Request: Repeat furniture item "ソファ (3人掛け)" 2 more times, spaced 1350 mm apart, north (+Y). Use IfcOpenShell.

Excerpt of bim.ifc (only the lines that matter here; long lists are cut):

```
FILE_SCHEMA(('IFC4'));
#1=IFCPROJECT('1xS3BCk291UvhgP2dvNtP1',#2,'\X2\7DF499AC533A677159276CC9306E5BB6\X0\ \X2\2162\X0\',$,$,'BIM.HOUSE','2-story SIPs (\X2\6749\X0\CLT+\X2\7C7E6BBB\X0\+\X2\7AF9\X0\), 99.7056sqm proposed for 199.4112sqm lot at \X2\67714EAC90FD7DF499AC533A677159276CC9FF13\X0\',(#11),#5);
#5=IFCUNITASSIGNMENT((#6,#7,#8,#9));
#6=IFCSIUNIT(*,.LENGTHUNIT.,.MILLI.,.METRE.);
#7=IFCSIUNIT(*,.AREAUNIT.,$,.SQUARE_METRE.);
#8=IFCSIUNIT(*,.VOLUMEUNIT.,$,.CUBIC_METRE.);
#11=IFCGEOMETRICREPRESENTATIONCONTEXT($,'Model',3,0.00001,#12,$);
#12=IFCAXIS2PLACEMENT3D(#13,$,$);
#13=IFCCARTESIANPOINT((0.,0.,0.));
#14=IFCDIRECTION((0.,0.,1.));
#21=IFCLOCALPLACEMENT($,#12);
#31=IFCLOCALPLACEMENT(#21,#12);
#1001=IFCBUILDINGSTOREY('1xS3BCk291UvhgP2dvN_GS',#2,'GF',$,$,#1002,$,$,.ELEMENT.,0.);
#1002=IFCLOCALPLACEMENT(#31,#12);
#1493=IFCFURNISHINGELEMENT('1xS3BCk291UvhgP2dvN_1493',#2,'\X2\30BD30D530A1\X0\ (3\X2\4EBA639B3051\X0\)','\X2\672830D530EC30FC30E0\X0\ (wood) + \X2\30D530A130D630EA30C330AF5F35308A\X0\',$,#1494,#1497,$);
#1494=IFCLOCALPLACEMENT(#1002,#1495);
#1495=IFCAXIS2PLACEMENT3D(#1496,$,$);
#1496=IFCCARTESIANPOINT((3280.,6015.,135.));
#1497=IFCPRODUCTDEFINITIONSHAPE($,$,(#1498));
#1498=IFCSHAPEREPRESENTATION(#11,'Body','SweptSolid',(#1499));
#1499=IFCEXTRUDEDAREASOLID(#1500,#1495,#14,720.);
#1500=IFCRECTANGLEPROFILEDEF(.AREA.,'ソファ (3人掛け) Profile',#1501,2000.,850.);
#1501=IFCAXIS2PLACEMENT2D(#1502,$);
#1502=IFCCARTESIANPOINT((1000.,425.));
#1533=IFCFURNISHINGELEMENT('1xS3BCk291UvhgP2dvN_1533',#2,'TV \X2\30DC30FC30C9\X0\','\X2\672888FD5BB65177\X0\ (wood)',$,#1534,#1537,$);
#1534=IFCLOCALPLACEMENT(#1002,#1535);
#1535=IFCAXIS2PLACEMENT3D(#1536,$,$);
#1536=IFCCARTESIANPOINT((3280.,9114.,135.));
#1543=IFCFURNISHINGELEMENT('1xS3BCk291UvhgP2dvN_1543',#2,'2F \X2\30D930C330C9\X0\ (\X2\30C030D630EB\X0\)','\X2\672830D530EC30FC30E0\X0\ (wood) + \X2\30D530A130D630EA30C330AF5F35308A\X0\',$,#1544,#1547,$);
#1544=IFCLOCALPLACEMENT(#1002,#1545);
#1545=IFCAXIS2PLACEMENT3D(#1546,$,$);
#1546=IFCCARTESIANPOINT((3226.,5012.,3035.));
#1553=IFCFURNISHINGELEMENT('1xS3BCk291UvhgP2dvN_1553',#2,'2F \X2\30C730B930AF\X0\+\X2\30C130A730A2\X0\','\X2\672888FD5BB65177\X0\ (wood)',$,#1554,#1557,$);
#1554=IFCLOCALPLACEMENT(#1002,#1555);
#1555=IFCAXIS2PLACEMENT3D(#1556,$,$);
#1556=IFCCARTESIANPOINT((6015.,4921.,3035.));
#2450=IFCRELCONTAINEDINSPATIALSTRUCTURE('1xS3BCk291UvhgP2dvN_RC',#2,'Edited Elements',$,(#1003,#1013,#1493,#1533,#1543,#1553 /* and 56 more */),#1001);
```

```python
import numpy as np
import ifcopenshell
import ifcopenshell.api.geometry
import ifcopenshell.api.root
import ifcopenshell.util.element
import ifcopenshell.util.placement
import ifcopenshell.util.unit

model = ifcopenshell.open("bim.ifc")
unit_scale = ifcopenshell.util.unit.calculate_unit_scale(model)


def reuse_history(source, copy):
    """copy_class also copies each property set's owner history, people and application; keep the originals."""
    for rel in copy.IsDefinedBy:
        if rel.is_a("IfcRelDefinesByProperties") and (history := rel.RelatingPropertyDefinition.OwnerHistory):
            rel.RelatingPropertyDefinition.OwnerHistory = source.OwnerHistory
            ifcopenshell.util.element.remove_deep2(model, history)


source = model.by_id(1493)
base = ifcopenshell.util.placement.get_local_placement(source.ObjectPlacement)
step = np.array([0.0, 1.0, 0.0]) * 1.35 / unit_scale

for i in range(1, 3):
    copy = ifcopenshell.api.root.copy_class(model, product=source)
    copy.Representation = ifcopenshell.util.element.copy_deep(
        model, source.Representation, exclude=["IfcGeometricRepresentationContext", "IfcRepresentationMap"]
    )
    reuse_history(source, copy)
    matrix = base.copy()
    matrix[:3, 3] += i * step
    print("added at", matrix[:3, 3].round(3) + 0.0)
    ifcopenshell.api.geometry.edit_object_placement(model, product=copy, matrix=matrix, is_si=False)

model.write("bim_edited.ifc")
```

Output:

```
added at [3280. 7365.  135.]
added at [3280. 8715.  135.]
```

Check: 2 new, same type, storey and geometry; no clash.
